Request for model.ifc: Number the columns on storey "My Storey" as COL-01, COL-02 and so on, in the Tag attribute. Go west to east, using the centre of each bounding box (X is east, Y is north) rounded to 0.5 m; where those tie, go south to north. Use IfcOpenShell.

First a look at what the model holds.

```python
import ifcopenshell
import ifcopenshell.util.element
import ifcopenshell.util.placement

model = ifcopenshell.open("model.ifc")
print(model.schema)
storey = next(s for s in model.by_type("IfcBuildingStorey") if s.Name == "My Storey")
columns = [e for e in ifcopenshell.util.element.get_decomposition(storey) if e.is_a("IfcColumn")]
for e in sorted(columns, key=lambda e: e.id()):
    origin = ifcopenshell.util.placement.get_local_placement(e.ObjectPlacement)[:3, 3]
    print(e.id(), e.Tag, e.Name, origin.round(2) + 0.0, sep=" | ")
```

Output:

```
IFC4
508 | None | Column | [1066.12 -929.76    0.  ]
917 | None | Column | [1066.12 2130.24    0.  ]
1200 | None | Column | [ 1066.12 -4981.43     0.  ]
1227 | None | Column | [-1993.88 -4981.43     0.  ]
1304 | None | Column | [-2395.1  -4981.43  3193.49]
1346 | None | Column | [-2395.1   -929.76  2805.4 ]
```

```python
import ifcopenshell
import ifcopenshell.geom
import ifcopenshell.util.element
import ifcopenshell.util.shape

model = ifcopenshell.open("model.ifc")
settings = ifcopenshell.geom.settings()
settings.set("use-world-coords", True)


def centre(element):
    shape = ifcopenshell.geom.create_shape(settings, element)
    return ifcopenshell.util.shape.get_bbox_centroid(shape.geometry)


storey = next(s for s in model.by_type("IfcBuildingStorey") if s.Name == "My Storey")
columns = [e for e in ifcopenshell.util.element.get_decomposition(storey) if e.is_a("IfcColumn")]

# Insertion points can sit at a corner or the storey origin, so sort by the geometry (in metres).
centres = {e: centre(e) for e in columns}
columns.sort(key=lambda e: (round(centres[e][0] / 0.5), centres[e][1]))

for i, e in enumerate(columns, start=1):
    number = f"COL-{i:02d}"
    e.Tag = number
    print(e.id(), number)

model.write("model-out.ifc")
```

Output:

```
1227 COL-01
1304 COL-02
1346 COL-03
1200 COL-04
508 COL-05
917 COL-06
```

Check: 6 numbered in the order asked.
